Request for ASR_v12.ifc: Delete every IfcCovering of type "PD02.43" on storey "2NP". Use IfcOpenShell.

First a look at what the model holds.

```python
import ifcopenshell
import ifcopenshell.util.element

model = ifcopenshell.open("ASR_v12.ifc")
print(model.schema)
storey = next(s for s in model.by_type("IfcBuildingStorey") if s.Name == "2NP")
coverings = [e for e in ifcopenshell.util.element.get_decomposition(storey) if e.is_a("IfcCovering")]
seen = {}
for e in coverings:
    element_type = ifcopenshell.util.element.get_type(e)
    name = element_type.Name if element_type not in (None, e) else None
    seen[name] = seen.get(name, 0) + 1
for name, count in sorted(seen.items(), key=str):
    print(count, "x", name)
```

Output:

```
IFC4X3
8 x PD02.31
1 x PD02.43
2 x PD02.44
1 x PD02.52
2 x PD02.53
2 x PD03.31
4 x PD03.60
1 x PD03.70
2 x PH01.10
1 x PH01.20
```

```python
import ifcopenshell
import ifcopenshell.api.root
import ifcopenshell.util.element

model = ifcopenshell.open("ASR_v12.ifc")

storey = next(s for s in model.by_type("IfcBuildingStorey") if s.Name == "2NP")
coverings = [e for e in ifcopenshell.util.element.get_decomposition(storey) if e.is_a("IfcCovering")]
targets = [e for e in coverings if (t := ifcopenshell.util.element.get_type(e)) not in (None, e) and t.Name == "PD02.43"]

for e in targets:
    ifcopenshell.api.root.remove_product(model, product=e)
print(len(targets), "removed")

model.write("ASR_v12_edited.ifc")
```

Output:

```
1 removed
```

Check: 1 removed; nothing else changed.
